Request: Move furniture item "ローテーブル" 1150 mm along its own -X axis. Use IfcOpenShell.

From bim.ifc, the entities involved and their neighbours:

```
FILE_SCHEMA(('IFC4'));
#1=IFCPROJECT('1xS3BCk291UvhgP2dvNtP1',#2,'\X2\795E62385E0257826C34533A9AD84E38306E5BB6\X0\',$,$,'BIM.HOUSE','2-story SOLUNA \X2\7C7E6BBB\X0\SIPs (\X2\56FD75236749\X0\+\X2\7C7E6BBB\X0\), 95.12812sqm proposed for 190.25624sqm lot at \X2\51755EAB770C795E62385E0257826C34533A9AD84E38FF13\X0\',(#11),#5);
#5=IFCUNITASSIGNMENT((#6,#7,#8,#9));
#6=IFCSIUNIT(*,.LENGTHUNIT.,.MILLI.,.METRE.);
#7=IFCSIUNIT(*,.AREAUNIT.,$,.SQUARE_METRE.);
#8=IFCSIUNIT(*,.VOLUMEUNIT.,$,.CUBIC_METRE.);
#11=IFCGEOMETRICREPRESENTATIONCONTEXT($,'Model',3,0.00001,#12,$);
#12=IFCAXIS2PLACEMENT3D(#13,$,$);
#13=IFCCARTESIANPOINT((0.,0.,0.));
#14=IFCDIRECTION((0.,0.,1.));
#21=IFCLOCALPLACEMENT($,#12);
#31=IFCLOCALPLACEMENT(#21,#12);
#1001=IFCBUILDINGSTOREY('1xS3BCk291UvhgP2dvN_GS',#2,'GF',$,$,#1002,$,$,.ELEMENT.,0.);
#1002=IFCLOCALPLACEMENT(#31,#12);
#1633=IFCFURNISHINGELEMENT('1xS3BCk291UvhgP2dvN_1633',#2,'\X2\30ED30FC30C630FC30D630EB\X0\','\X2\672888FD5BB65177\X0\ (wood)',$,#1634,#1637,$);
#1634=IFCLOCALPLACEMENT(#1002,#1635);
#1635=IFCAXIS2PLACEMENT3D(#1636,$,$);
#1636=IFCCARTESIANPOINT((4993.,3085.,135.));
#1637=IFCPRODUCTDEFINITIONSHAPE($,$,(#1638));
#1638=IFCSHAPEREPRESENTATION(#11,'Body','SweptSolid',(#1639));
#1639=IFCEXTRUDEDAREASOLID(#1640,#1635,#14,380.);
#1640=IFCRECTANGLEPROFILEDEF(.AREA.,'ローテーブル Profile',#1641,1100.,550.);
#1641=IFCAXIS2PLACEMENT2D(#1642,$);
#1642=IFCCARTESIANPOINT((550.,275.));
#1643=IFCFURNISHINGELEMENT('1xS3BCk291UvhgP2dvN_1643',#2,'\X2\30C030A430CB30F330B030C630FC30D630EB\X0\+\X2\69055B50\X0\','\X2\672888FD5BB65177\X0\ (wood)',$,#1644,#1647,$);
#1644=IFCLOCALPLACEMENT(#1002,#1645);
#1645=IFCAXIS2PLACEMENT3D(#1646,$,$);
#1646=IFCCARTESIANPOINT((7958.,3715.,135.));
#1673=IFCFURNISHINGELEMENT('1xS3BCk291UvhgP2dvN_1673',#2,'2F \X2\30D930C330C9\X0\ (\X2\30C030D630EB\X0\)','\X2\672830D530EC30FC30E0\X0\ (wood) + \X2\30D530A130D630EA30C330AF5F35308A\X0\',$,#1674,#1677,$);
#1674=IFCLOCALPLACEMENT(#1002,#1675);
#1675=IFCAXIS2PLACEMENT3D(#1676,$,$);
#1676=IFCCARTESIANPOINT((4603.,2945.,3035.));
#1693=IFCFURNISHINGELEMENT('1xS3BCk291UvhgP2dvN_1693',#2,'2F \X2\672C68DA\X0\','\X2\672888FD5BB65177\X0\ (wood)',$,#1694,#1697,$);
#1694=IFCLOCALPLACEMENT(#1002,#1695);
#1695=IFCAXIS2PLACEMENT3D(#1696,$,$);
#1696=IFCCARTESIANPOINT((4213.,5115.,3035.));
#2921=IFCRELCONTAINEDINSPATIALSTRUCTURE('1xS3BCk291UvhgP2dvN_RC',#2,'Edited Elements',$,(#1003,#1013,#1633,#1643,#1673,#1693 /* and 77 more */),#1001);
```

```python
import ifcopenshell
import ifcopenshell.api.geometry
import ifcopenshell.util.placement

model = ifcopenshell.open("bim.ifc")

item = model.by_guid("1xS3BCk291UvhgP2dvN_1633")
matrix = ifcopenshell.util.placement.get_local_placement(item.ObjectPlacement)
matrix[:3, 3] -= matrix[:3, 0] * 1150.0
ifcopenshell.api.geometry.edit_object_placement(model, product=item, matrix=matrix, is_si=False)

print(ifcopenshell.util.placement.get_local_placement(item.ObjectPlacement).round(3) + 0.0)

model.write("bim_rev.ifc")
```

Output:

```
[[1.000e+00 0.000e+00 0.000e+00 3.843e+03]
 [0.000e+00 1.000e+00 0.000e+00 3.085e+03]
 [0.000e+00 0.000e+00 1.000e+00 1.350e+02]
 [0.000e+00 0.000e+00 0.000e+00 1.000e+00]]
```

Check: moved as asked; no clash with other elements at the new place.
